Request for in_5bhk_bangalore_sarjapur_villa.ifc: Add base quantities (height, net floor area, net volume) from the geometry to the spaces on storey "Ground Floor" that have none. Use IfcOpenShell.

First a look at what the model holds.

```python
import ifcopenshell
import ifcopenshell.util.element
import ifcopenshell.util.unit

model = ifcopenshell.open("in_5bhk_bangalore_sarjapur_villa.ifc")
print(model.schema)
for unit_type in ("LENGTHUNIT", "AREAUNIT", "VOLUMEUNIT"):
    print(unit_type, ifcopenshell.util.unit.calculate_unit_scale(model, unit_type))
storey = next(s for s in model.by_type("IfcBuildingStorey") if s.Name == "Ground Floor")
spaces = [e for e in ifcopenshell.util.element.get_decomposition(storey) if e.is_a("IfcSpace")]
for e in sorted(spaces, key=lambda e: e.id()):
    print(e.id(), e.is_a(), e.Name, list(ifcopenshell.util.element.get_psets(e, qtos_only=True)), sep=" | ")
```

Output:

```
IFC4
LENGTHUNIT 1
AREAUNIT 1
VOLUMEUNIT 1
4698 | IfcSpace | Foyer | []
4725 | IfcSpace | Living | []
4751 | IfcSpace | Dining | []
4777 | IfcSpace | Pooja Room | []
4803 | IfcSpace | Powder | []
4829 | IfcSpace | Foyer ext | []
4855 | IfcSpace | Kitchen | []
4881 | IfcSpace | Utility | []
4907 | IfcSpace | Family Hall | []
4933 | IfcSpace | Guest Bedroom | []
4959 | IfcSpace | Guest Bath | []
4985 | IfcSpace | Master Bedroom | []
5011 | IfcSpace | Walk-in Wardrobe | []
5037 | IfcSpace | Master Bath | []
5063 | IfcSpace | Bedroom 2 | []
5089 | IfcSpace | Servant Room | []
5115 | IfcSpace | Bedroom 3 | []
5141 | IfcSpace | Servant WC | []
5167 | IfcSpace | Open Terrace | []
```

```python
import ifcopenshell
import ifcopenshell.api.pset
import ifcopenshell.geom
import ifcopenshell.util.element
import ifcopenshell.util.shape
import ifcopenshell.util.unit

model = ifcopenshell.open("in_5bhk_bangalore_sarjapur_villa.ifc")
unit_scale = ifcopenshell.util.unit.calculate_unit_scale(model)
area_scale = ifcopenshell.util.unit.calculate_unit_scale(model, "AREAUNIT")
volume_scale = ifcopenshell.util.unit.calculate_unit_scale(model, "VOLUMEUNIT")
settings = ifcopenshell.geom.settings()

storey = next(s for s in model.by_type("IfcBuildingStorey") if s.Name == "Ground Floor")
spaces = [e for e in ifcopenshell.util.element.get_decomposition(storey) if e.is_a("IfcSpace")]

for e in sorted(spaces, key=lambda e: e.id()):
    if ifcopenshell.util.element.get_psets(e, qtos_only=True, should_inherit=False):
        continue
    # Geometry comes back in metres, in the element's own axes.
    shape = ifcopenshell.geom.create_shape(settings, e)
    values = {
        "Height": ifcopenshell.util.shape.get_z(shape.geometry) / unit_scale,
        "NetFloorArea": ifcopenshell.util.shape.get_footprint_area(shape.geometry) / area_scale,
        "NetVolume": ifcopenshell.util.shape.get_volume(shape.geometry) / volume_scale,
    }
    qto = ifcopenshell.api.pset.add_qto(model, product=e, name="Qto_SpaceBaseQuantities")
    ifcopenshell.api.pset.edit_qto(model, qto=qto, properties=values)
    print(e.id(), {k: round(v, 3) for k, v in values.items()})

model.write("in_5bhk_bangalore_sarjapur_villa_edited.ifc")
```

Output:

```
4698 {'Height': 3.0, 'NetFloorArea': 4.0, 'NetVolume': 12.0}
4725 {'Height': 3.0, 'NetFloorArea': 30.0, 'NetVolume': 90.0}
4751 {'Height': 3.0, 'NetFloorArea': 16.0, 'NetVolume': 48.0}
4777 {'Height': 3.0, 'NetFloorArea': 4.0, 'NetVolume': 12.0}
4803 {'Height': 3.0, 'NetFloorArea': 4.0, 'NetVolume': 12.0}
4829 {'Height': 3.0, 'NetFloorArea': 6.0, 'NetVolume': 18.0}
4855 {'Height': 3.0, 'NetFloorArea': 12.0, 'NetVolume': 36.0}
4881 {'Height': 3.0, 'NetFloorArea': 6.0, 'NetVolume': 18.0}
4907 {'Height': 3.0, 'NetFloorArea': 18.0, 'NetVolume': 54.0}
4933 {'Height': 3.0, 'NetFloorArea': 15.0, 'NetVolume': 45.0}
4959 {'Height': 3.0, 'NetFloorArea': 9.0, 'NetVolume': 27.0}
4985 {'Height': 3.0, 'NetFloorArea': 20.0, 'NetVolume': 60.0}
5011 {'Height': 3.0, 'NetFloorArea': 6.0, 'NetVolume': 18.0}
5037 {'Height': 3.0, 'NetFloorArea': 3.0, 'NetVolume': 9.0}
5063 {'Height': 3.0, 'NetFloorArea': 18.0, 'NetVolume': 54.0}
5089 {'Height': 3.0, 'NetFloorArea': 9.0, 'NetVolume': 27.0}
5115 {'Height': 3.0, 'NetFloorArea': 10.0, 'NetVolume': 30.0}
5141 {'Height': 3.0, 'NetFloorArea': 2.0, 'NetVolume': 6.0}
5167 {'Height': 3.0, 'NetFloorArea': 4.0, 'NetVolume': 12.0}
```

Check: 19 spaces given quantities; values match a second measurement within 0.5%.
